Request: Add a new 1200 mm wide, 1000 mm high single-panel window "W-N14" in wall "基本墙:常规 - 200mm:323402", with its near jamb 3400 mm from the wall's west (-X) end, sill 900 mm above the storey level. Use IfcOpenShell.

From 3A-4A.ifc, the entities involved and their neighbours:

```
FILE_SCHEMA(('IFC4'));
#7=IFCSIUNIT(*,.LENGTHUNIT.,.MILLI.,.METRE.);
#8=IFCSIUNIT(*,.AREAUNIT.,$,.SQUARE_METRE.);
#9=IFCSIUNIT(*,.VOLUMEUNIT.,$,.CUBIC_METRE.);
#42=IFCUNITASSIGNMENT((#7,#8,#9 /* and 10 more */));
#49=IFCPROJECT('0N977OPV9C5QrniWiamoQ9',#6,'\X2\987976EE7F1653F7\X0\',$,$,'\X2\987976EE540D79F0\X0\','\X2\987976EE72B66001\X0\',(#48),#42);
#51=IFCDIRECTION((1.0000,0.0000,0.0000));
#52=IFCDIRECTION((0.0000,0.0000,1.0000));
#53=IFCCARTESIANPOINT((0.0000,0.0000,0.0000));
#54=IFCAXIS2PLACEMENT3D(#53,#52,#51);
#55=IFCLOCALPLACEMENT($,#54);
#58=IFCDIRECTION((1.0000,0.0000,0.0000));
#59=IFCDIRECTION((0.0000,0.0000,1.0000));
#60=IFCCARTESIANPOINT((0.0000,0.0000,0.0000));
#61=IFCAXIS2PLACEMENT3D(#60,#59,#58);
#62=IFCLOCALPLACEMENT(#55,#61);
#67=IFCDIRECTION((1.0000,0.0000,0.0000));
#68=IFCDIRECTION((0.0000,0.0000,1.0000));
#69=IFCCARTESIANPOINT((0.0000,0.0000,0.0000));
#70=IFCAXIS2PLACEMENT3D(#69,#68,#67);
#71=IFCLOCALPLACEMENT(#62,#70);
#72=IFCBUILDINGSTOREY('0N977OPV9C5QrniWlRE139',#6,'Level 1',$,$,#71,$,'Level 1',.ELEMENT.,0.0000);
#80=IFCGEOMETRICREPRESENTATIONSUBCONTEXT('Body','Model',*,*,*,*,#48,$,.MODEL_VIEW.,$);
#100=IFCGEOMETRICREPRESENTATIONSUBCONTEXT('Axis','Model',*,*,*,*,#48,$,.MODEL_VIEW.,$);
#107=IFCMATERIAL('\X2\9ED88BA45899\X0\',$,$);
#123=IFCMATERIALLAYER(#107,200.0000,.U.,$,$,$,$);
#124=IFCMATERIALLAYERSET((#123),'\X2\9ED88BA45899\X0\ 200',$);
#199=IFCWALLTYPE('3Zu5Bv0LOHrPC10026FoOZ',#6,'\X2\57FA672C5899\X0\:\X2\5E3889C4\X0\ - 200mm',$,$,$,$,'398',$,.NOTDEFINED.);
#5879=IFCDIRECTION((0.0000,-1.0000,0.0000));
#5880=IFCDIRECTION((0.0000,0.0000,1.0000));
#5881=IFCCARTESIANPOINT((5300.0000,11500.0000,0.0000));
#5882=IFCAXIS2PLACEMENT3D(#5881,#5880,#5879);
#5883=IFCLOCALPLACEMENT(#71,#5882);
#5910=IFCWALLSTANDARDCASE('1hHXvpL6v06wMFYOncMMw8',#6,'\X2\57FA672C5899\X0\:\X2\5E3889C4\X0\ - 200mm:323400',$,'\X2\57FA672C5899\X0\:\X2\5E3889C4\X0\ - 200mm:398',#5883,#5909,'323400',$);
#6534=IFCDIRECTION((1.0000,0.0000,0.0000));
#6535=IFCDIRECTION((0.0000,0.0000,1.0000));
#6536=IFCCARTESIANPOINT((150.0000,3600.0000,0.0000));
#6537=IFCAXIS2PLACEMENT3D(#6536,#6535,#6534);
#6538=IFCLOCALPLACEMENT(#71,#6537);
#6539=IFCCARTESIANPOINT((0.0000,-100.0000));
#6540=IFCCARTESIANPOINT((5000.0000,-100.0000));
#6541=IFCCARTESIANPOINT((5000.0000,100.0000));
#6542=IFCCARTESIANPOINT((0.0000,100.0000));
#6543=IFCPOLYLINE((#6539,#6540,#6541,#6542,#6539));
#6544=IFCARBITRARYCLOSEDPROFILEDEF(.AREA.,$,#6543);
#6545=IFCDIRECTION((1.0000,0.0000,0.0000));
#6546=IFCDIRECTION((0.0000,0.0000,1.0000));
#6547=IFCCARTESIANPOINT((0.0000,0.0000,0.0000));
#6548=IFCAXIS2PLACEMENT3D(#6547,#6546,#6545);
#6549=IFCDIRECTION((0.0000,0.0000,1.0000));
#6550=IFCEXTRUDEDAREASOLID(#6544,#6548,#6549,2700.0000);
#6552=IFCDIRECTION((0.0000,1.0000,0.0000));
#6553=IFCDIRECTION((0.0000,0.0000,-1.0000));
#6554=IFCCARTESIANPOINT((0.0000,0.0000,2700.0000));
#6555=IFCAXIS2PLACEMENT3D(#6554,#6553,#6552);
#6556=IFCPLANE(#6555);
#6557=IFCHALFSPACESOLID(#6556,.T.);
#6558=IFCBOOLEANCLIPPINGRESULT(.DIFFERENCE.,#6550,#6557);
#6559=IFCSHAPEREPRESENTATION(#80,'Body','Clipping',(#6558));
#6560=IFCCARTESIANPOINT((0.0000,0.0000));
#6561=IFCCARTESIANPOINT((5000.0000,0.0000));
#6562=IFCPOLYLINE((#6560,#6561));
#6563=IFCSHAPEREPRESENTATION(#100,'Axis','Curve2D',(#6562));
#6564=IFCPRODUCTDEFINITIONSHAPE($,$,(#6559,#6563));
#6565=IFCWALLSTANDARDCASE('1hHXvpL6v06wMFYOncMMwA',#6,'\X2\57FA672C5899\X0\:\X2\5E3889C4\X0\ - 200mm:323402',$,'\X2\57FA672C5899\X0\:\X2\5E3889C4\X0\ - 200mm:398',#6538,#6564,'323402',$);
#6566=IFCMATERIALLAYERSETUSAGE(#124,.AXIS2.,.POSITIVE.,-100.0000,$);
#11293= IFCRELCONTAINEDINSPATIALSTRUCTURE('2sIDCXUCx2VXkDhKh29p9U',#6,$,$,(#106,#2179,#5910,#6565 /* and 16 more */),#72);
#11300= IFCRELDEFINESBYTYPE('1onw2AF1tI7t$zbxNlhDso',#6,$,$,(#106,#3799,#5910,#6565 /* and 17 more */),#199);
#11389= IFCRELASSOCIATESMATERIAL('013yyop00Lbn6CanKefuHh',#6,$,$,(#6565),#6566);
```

```python
import numpy as np
import ifcopenshell
import ifcopenshell.api.feature
import ifcopenshell.api.geometry
import ifcopenshell.api.root
import ifcopenshell.api.spatial
import ifcopenshell.geom
import ifcopenshell.util.element
import ifcopenshell.util.placement
import ifcopenshell.util.representation
import ifcopenshell.util.shape
import ifcopenshell.util.unit

model = ifcopenshell.open("3A-4A.ifc")
unit_scale = ifcopenshell.util.unit.calculate_unit_scale(model)
settings = ifcopenshell.geom.settings()


def volume(element):
    """Net volume in cubic metres, openings subtracted."""
    shape = ifcopenshell.geom.create_shape(settings, element)
    return ifcopenshell.util.shape.get_volume(shape.geometry)


wall = model.by_guid("1hHXvpL6v06wMFYOncMMwA")
storey = ifcopenshell.util.element.get_container(wall, ifc_class="IfcBuildingStorey")
context = ifcopenshell.util.representation.get_context(model, "Model", "Body", "MODEL_VIEW")
before = volume(wall)

width, height, from_end, sill = 1.2, 1, 3.4, 0.9  # metres

# The wall runs along its own X axis, and the end named is its -X end.
wall_shape = ifcopenshell.geom.create_shape(settings, wall)
x, y, z = ifcopenshell.util.shape.get_vertices(wall_shape.geometry).T
start = x.min() + from_end
face, thickness = float(y.min()), float(y.max() - y.min())
wall_matrix = ifcopenshell.util.placement.get_local_placement(wall.ObjectPlacement)
level = ifcopenshell.util.placement.get_local_placement(storey.ObjectPlacement)[2, 3]


def in_wall(x, y):
    """Placement at x, y metres in the wall's axes, at sill height."""
    matrix = wall_matrix.copy()
    matrix[:, 3] = wall_matrix @ np.array([x / unit_scale, y / unit_scale, 0.0, 1.0])
    matrix[2, 3] = level + sill / unit_scale
    return matrix


# Opening: a box that overshoots both wall faces by 50 mm.
opening = ifcopenshell.api.root.create_entity(model, ifc_class="IfcOpeningElement", predefined_type="OPENING")
box = ifcopenshell.api.geometry.add_wall_representation(
    model, context=context, length=width, height=height, thickness=thickness + 0.1
)
ifcopenshell.api.geometry.assign_representation(model, product=opening, representation=box)
ifcopenshell.api.geometry.edit_object_placement(model, product=opening, matrix=in_wall(start, face - 0.05), is_si=False)
ifcopenshell.api.feature.add_feature(model, feature=opening, element=wall)

window = ifcopenshell.api.root.create_entity(model, ifc_class="IfcWindow", name="W-N14", predefined_type="WINDOW")
window.OverallWidth, window.OverallHeight = width / unit_scale, height / unit_scale
window.PartitioningType = "SINGLE_PANEL"
body = ifcopenshell.api.geometry.add_window_representation(
    model,
    context=context,
    overall_width=window.OverallWidth,
    overall_height=window.OverallHeight,
    partition_type="SINGLE_PANEL",
)
ifcopenshell.api.geometry.assign_representation(model, product=window, representation=body)
ifcopenshell.api.spatial.assign_container(model, products=[window], relating_structure=storey)
ifcopenshell.api.feature.add_filling(model, opening=opening, element=window)

# Centre the window in the wall's thickness.
ifcopenshell.api.geometry.edit_object_placement(model, product=window, matrix=in_wall(start, face), is_si=False)
window_shape = ifcopenshell.geom.create_shape(settings, window)
depth = ifcopenshell.util.shape.get_vertices(window_shape.geometry)[:, 1]
offset = face + thickness / 2 - (depth.min() + depth.max()) / 2
ifcopenshell.api.geometry.edit_object_placement(model, product=window, matrix=in_wall(start, offset), is_si=False)

after = volume(wall)

print(f"wall volume {before:.3f} -> {after:.3f} m3")

model.write("3A-4A_rev.ifc")
```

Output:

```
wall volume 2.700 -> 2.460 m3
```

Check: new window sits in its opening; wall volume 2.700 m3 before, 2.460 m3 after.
